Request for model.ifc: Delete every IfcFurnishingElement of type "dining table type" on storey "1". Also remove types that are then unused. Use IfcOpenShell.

First a look at what the model holds.

```python
import ifcopenshell
import ifcopenshell.util.element

model = ifcopenshell.open("model.ifc")
print(model.schema)
storey = next(s for s in model.by_type("IfcBuildingStorey") if s.Name == "1")
furniture = [e for e in ifcopenshell.util.element.get_decomposition(storey) if e.is_a("IfcFurnishingElement")]
seen = {}
for e in furniture:
    element_type = ifcopenshell.util.element.get_type(e)
    name = element_type.Name if element_type not in (None, e) else None
    seen[name] = seen.get(name, 0) + 1
for name, count in sorted(seen.items(), key=str):
    print(count, "x", name)
```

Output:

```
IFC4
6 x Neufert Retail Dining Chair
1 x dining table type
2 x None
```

```python
import ifcopenshell
import ifcopenshell.api.root
import ifcopenshell.util.element

model = ifcopenshell.open("model.ifc")

storey = next(s for s in model.by_type("IfcBuildingStorey") if s.Name == "1")
furniture = [e for e in ifcopenshell.util.element.get_decomposition(storey) if e.is_a("IfcFurnishingElement")]
targets = [e for e in furniture if (t := ifcopenshell.util.element.get_type(e)) not in (None, e) and t.Name == "dining table type"]
types = {ifcopenshell.util.element.get_type(e) for e in targets} - {None, *targets}

for e in targets:
    ifcopenshell.api.root.remove_product(model, product=e)
print(len(targets), "removed")

unused = [t for t in types if not ifcopenshell.util.element.get_types(t)]
for t in unused:
    ifcopenshell.api.root.remove_product(model, product=t)
print(len(unused), "unused types removed")

model.write("model_edited.ifc")
```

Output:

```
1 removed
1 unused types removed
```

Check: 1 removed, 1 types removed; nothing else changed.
